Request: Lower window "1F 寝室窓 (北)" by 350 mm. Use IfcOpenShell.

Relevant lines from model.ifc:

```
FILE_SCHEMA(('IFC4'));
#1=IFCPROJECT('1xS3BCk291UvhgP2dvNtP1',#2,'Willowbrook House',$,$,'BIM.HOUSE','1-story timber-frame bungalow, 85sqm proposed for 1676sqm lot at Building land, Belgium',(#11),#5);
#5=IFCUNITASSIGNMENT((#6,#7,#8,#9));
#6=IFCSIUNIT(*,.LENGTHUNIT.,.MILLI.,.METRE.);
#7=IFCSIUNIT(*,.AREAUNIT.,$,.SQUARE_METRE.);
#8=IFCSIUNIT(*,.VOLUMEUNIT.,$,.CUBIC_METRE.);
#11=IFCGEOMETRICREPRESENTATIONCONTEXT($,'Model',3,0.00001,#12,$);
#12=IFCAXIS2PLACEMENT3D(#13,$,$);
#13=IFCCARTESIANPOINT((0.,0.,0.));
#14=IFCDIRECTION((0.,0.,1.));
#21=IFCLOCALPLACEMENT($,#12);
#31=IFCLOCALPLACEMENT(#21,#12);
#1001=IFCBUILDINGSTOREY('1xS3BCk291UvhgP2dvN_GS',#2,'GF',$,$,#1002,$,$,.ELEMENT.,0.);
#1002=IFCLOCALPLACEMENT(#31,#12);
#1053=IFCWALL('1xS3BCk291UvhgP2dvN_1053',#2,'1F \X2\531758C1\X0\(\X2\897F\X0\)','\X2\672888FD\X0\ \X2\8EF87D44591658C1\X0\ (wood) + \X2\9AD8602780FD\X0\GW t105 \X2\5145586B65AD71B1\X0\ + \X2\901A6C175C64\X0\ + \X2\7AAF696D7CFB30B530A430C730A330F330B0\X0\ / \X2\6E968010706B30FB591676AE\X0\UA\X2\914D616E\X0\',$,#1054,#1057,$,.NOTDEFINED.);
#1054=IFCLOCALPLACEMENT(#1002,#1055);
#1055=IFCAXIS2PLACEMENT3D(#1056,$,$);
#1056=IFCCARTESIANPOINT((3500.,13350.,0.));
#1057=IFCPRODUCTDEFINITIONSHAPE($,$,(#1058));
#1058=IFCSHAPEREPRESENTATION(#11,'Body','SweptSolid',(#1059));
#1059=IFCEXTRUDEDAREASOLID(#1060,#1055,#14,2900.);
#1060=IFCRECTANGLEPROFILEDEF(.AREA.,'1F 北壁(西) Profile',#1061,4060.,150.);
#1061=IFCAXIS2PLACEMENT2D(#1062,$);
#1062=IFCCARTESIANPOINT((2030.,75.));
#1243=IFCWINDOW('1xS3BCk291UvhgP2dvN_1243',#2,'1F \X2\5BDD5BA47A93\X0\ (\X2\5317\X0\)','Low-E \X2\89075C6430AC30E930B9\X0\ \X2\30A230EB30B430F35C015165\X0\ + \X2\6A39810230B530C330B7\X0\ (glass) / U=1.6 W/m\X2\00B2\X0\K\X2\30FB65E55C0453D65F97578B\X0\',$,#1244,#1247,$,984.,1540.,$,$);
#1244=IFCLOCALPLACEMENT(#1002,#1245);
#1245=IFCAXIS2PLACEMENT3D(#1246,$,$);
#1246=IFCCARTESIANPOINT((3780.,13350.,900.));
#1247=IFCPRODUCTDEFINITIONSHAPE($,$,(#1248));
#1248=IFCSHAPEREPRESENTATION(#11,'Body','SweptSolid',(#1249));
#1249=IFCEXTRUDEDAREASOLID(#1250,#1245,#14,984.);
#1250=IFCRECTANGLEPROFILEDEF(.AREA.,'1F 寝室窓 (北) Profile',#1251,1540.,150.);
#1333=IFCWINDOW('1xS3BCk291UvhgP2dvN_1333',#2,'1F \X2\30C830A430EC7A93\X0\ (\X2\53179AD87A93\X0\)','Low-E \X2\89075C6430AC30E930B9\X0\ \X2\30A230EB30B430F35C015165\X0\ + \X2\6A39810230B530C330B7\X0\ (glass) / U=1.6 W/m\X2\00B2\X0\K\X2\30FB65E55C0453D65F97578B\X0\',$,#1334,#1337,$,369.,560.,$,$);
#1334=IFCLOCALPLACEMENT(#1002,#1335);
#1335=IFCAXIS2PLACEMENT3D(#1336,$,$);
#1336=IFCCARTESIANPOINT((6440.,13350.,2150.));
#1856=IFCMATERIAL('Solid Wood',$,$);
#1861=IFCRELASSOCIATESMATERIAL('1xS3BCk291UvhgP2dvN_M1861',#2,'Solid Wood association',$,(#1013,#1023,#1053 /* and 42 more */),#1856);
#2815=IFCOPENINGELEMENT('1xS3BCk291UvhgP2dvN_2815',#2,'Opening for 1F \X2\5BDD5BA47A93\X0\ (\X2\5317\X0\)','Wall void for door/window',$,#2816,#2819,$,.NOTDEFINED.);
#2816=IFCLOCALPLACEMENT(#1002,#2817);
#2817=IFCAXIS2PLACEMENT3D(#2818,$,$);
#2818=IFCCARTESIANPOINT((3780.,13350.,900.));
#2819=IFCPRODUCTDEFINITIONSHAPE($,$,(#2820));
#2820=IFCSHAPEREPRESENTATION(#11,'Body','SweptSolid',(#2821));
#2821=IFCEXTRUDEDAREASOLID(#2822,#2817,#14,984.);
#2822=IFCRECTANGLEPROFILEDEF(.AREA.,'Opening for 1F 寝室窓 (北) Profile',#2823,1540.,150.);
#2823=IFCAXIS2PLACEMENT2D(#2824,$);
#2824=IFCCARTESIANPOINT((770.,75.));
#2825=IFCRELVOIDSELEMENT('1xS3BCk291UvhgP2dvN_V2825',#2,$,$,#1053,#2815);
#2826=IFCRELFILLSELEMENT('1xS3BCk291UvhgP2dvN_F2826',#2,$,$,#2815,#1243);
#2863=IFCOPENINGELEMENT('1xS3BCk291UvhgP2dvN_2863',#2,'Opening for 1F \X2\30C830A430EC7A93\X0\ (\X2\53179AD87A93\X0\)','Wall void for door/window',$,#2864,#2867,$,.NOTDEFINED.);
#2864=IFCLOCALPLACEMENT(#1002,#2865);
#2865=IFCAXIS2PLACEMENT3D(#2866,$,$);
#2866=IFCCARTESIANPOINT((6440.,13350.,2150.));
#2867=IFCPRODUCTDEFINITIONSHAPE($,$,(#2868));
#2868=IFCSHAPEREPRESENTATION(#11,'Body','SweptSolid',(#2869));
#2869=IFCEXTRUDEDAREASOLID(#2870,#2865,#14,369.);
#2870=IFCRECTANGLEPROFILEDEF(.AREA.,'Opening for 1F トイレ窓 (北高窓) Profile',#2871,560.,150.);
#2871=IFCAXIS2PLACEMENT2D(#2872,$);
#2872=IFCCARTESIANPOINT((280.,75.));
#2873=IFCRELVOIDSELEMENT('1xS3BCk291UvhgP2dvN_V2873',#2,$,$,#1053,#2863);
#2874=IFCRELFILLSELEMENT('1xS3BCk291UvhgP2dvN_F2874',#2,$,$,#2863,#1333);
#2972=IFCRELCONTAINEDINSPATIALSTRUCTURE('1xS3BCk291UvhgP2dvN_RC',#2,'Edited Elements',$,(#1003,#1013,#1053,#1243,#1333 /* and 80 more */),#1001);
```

```python
import numpy as np
import ifcopenshell
import ifcopenshell.api.geometry
import ifcopenshell.util.placement
import ifcopenshell.util.unit

model = ifcopenshell.open("model.ifc")
unit_scale = ifcopenshell.util.unit.calculate_unit_scale(model)

window = model.by_guid("1xS3BCk291UvhgP2dvN_1243")
opening = window.FillsVoids[0].RelatingOpeningElement
dz = -0.35 / unit_scale

shift = np.array([0.0, 0.0, dz])
# The window is not placed relative to its opening, so move both.
for product in (opening, window):
    matrix = ifcopenshell.util.placement.get_local_placement(product.ObjectPlacement)
    matrix[:3, 3] += shift
    ifcopenshell.api.geometry.edit_object_placement(model, product=product, matrix=matrix, is_si=False)

print(f"moved by {dz * unit_scale:+.3f} m")

model.write("model-out.ifc")
```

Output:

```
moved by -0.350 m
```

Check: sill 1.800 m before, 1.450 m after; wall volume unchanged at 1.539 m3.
